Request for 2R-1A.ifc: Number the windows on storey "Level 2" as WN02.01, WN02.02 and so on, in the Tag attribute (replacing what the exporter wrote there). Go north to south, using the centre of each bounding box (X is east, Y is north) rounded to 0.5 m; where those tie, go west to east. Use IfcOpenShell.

First a look at what the model holds.

```python
import ifcopenshell
import ifcopenshell.util.element
import ifcopenshell.util.placement

model = ifcopenshell.open("2R-1A.ifc")
print(model.schema)
storey = next(s for s in model.by_type("IfcBuildingStorey") if s.Name == "Level 2")
windows = [e for e in ifcopenshell.util.element.get_decomposition(storey) if e.is_a("IfcWindow")]
for e in sorted(windows, key=lambda e: e.id()):
    origin = ifcopenshell.util.placement.get_local_placement(e.ObjectPlacement)[:3, 3]
    print(e.id(), e.Tag, e.Name, origin.round(2) + 0.0, sep=" | ")
```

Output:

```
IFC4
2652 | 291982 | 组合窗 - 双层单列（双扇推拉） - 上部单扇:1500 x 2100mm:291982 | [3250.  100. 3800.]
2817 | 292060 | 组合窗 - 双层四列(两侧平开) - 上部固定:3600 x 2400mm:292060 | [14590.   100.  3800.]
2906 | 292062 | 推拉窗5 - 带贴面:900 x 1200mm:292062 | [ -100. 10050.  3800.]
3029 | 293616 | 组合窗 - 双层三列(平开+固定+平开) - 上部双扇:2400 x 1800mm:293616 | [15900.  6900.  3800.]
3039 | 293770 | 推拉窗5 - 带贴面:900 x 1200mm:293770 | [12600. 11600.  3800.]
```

```python
import ifcopenshell
import ifcopenshell.geom
import ifcopenshell.util.element
import ifcopenshell.util.shape

model = ifcopenshell.open("2R-1A.ifc")
settings = ifcopenshell.geom.settings()
settings.set("use-world-coords", True)


def centre(element):
    shape = ifcopenshell.geom.create_shape(settings, element)
    return ifcopenshell.util.shape.get_bbox_centroid(shape.geometry)


storey = next(s for s in model.by_type("IfcBuildingStorey") if s.Name == "Level 2")
windows = [e for e in ifcopenshell.util.element.get_decomposition(storey) if e.is_a("IfcWindow")]

# Insertion points can sit at a corner or the storey origin, so sort by the geometry (in metres).
centres = {e: centre(e) for e in windows}
windows.sort(key=lambda e: (-round(centres[e][1] / 0.5), centres[e][0]))

for i, e in enumerate(windows, start=1):
    number = f"WN02.{i:02d}"
    e.Tag = number
    print(e.id(), number)

model.write("2R-1A_updated.ifc")
```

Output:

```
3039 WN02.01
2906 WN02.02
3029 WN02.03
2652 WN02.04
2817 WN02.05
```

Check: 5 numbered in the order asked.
